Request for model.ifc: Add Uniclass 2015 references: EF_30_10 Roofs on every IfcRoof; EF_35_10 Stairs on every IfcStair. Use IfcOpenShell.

First a look at what the model holds.

```python
import ifcopenshell

model = ifcopenshell.open("model.ifc")
print(model.schema)
print("classifications:", [c.Name for c in model.by_type("IfcClassification")])
for ifc_class in ("IfcDoor", "IfcRoof", "IfcStair", "IfcWall", "IfcWindow"):
    print(ifc_class, len(model.by_type(ifc_class)))
```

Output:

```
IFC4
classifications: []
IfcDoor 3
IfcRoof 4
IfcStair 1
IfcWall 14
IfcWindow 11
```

```python
import ifcopenshell
import ifcopenshell.api.classification

model = ifcopenshell.open("model.ifc")

system = ifcopenshell.api.classification.add_classification(model, classification="Uniclass 2015")

codes = {
    "IfcRoof": ("EF_30_10", "Roofs"),
    "IfcStair": ("EF_35_10", "Stairs"),
}
for ifc_class, (code, name) in codes.items():
    products = model.by_type(ifc_class)
    ifcopenshell.api.classification.add_reference(
        model, products=products, classification=system, identification=code, name=name
    )
    print(code, len(products))

model.write("model-out.ifc")
```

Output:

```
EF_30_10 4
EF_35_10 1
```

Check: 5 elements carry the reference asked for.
